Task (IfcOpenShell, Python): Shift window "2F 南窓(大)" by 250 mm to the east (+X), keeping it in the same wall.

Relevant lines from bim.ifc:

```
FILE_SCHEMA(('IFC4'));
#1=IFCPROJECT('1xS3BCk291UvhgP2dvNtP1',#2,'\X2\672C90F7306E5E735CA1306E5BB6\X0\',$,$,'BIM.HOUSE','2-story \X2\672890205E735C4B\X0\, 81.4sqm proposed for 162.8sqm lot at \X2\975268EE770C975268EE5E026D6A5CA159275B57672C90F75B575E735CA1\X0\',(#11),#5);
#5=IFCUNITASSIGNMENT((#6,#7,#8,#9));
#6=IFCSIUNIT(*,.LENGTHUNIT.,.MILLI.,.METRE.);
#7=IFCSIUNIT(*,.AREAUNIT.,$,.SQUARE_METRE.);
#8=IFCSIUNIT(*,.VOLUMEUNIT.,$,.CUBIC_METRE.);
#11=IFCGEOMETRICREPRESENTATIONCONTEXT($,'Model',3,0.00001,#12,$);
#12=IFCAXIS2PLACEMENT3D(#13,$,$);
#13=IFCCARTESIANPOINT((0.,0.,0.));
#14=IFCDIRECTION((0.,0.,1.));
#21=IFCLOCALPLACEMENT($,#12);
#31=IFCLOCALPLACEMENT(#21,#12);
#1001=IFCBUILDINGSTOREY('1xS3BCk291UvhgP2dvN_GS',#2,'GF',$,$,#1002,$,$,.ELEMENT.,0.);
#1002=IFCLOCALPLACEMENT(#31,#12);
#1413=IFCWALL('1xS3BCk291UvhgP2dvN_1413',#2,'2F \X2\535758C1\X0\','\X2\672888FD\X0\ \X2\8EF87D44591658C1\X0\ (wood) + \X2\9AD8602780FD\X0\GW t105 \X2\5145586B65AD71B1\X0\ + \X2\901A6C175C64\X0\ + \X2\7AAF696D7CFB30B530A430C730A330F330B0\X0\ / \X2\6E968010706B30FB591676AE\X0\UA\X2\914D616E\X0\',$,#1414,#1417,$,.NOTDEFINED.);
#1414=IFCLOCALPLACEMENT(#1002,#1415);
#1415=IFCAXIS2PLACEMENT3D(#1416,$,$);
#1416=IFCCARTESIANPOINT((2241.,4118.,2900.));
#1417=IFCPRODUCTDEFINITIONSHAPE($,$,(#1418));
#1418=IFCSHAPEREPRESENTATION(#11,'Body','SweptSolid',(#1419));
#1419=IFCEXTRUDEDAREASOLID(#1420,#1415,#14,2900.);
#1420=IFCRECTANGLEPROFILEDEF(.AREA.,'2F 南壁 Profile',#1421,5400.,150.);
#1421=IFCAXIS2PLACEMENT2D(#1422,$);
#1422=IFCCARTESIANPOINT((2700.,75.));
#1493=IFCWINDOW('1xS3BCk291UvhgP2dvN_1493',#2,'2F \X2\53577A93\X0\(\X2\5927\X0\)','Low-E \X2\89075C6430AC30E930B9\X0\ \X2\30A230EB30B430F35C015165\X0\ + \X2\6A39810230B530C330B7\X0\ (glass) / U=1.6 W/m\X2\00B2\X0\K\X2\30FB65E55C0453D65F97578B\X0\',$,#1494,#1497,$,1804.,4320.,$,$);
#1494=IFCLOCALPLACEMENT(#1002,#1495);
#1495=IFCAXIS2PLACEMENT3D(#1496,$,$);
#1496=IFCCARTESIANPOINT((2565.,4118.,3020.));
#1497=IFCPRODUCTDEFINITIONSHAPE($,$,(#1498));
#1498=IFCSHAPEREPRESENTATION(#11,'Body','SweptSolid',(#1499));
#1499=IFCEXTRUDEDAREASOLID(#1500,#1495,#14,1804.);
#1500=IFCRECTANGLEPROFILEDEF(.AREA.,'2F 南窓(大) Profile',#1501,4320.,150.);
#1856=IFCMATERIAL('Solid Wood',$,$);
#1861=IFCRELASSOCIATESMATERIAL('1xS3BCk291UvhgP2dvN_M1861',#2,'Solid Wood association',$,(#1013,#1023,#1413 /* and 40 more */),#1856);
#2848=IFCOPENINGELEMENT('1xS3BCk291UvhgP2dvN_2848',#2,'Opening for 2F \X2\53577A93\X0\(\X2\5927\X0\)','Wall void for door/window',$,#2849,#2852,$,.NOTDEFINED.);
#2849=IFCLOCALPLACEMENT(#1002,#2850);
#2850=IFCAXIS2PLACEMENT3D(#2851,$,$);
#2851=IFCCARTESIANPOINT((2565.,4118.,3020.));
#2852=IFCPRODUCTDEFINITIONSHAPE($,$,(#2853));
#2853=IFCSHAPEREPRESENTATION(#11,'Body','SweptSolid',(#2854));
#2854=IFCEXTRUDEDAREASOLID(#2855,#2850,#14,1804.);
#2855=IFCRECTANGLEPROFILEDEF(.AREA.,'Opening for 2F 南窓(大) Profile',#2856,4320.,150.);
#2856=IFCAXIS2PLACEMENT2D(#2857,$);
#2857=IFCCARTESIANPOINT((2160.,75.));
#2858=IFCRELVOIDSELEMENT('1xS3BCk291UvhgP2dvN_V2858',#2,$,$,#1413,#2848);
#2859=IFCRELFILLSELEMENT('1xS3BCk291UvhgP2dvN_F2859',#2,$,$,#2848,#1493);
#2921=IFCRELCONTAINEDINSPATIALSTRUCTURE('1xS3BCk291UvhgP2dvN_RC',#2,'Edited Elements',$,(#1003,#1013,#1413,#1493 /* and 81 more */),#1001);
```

```python
import ifcopenshell
import ifcopenshell.api.geometry
import ifcopenshell.util.placement
import ifcopenshell.util.unit

model = ifcopenshell.open("bim.ifc")
unit_scale = ifcopenshell.util.unit.calculate_unit_scale(model)

window = model.by_guid("1xS3BCk291UvhgP2dvN_1493")
opening = window.FillsVoids[0].RelatingOpeningElement
wall = opening.VoidsElements[0].RelatingBuildingElement

wall_matrix = ifcopenshell.util.placement.get_local_placement(wall.ObjectPlacement)
shift = wall_matrix[:3, 0] * 0.25 / unit_scale
before = ifcopenshell.util.placement.get_local_placement(window.ObjectPlacement)[:3, 3].copy()

# The window is not placed relative to its opening, so move both.
for product in (opening, window):
    matrix = ifcopenshell.util.placement.get_local_placement(product.ObjectPlacement)
    matrix[:3, 3] += shift
    ifcopenshell.api.geometry.edit_object_placement(model, product=product, matrix=matrix, is_si=False)

after = ifcopenshell.util.placement.get_local_placement(window.ObjectPlacement)[:3, 3]
print("window moved by", (after - before).round(3) + 0.0)

model.write("bim_v2.ifc")
```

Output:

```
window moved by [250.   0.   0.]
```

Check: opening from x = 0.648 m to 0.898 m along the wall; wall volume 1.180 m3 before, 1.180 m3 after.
